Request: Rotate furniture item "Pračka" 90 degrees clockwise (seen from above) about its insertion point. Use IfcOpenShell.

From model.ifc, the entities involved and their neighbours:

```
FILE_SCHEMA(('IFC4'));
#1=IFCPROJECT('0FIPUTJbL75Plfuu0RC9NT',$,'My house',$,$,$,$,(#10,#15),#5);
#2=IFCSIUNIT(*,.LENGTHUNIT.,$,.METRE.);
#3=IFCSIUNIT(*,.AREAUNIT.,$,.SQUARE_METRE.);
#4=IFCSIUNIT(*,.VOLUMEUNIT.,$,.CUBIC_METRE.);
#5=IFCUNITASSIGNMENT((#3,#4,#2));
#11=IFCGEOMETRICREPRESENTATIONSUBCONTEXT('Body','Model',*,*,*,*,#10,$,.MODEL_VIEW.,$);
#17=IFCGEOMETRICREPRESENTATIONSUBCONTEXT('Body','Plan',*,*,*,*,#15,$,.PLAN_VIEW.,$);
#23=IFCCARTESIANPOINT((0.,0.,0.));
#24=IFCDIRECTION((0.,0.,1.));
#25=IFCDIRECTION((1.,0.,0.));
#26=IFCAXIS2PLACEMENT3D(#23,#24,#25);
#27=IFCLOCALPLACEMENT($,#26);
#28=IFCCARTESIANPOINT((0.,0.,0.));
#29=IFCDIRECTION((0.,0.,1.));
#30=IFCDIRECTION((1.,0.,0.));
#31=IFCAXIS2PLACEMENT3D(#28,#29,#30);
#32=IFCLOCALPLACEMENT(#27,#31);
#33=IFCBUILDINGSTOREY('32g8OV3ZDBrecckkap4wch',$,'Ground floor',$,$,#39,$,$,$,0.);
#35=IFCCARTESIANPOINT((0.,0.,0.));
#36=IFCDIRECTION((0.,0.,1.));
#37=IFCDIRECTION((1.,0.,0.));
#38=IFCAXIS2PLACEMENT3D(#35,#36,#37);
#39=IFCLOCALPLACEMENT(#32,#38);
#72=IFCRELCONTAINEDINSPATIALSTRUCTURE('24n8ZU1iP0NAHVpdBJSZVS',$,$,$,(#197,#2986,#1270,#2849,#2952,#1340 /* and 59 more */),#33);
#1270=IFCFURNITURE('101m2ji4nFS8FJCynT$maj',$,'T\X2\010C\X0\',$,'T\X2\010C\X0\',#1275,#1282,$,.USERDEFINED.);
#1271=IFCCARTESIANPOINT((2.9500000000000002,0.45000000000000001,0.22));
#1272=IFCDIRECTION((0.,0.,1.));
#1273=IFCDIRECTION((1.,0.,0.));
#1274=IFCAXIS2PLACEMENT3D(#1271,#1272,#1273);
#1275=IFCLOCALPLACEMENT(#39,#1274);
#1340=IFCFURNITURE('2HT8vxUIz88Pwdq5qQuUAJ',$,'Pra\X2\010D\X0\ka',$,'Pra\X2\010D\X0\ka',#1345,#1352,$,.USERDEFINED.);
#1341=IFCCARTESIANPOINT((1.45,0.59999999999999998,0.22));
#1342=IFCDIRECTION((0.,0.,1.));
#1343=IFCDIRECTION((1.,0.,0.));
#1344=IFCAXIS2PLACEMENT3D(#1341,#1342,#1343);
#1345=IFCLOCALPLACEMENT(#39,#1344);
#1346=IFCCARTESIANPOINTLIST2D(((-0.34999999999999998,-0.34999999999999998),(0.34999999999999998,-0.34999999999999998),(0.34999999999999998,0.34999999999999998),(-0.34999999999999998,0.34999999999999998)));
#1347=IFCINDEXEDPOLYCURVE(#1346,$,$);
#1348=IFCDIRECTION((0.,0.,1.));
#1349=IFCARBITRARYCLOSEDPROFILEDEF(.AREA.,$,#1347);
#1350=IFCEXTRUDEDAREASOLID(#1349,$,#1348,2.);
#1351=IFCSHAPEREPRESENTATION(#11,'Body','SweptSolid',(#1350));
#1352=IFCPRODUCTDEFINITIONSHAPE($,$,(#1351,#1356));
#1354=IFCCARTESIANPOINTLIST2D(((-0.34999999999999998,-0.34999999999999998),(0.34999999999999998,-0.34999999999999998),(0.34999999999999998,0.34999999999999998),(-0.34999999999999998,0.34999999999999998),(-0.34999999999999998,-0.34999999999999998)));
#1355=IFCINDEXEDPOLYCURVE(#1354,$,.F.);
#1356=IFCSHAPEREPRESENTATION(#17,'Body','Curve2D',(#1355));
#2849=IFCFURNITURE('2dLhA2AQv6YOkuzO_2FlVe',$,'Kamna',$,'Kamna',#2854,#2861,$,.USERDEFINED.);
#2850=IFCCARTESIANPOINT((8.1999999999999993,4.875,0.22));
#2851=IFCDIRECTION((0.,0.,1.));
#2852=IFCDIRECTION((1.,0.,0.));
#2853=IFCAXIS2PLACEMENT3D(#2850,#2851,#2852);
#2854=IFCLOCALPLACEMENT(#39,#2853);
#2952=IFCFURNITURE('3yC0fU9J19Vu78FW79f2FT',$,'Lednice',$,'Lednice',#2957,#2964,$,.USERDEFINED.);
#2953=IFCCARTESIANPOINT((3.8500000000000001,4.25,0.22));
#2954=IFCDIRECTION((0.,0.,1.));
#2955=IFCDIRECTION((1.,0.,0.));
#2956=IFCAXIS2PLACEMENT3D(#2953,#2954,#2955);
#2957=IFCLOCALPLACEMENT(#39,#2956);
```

```python
import ifcopenshell
import ifcopenshell.api.geometry
import ifcopenshell.util.placement

model = ifcopenshell.open("model.ifc")

item = model.by_id(1340)
matrix = ifcopenshell.util.placement.get_local_placement(item.ObjectPlacement)
matrix = matrix @ ifcopenshell.util.placement.rotation(-90, "Z")
ifcopenshell.api.geometry.edit_object_placement(model, product=item, matrix=matrix, is_si=False)

print(ifcopenshell.util.placement.get_local_placement(item.ObjectPlacement).round(3) + 0.0)

model.write("model_rev.ifc")
```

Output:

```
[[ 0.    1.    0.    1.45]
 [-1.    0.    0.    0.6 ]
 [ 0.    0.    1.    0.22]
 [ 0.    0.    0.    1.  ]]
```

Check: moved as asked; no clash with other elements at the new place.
